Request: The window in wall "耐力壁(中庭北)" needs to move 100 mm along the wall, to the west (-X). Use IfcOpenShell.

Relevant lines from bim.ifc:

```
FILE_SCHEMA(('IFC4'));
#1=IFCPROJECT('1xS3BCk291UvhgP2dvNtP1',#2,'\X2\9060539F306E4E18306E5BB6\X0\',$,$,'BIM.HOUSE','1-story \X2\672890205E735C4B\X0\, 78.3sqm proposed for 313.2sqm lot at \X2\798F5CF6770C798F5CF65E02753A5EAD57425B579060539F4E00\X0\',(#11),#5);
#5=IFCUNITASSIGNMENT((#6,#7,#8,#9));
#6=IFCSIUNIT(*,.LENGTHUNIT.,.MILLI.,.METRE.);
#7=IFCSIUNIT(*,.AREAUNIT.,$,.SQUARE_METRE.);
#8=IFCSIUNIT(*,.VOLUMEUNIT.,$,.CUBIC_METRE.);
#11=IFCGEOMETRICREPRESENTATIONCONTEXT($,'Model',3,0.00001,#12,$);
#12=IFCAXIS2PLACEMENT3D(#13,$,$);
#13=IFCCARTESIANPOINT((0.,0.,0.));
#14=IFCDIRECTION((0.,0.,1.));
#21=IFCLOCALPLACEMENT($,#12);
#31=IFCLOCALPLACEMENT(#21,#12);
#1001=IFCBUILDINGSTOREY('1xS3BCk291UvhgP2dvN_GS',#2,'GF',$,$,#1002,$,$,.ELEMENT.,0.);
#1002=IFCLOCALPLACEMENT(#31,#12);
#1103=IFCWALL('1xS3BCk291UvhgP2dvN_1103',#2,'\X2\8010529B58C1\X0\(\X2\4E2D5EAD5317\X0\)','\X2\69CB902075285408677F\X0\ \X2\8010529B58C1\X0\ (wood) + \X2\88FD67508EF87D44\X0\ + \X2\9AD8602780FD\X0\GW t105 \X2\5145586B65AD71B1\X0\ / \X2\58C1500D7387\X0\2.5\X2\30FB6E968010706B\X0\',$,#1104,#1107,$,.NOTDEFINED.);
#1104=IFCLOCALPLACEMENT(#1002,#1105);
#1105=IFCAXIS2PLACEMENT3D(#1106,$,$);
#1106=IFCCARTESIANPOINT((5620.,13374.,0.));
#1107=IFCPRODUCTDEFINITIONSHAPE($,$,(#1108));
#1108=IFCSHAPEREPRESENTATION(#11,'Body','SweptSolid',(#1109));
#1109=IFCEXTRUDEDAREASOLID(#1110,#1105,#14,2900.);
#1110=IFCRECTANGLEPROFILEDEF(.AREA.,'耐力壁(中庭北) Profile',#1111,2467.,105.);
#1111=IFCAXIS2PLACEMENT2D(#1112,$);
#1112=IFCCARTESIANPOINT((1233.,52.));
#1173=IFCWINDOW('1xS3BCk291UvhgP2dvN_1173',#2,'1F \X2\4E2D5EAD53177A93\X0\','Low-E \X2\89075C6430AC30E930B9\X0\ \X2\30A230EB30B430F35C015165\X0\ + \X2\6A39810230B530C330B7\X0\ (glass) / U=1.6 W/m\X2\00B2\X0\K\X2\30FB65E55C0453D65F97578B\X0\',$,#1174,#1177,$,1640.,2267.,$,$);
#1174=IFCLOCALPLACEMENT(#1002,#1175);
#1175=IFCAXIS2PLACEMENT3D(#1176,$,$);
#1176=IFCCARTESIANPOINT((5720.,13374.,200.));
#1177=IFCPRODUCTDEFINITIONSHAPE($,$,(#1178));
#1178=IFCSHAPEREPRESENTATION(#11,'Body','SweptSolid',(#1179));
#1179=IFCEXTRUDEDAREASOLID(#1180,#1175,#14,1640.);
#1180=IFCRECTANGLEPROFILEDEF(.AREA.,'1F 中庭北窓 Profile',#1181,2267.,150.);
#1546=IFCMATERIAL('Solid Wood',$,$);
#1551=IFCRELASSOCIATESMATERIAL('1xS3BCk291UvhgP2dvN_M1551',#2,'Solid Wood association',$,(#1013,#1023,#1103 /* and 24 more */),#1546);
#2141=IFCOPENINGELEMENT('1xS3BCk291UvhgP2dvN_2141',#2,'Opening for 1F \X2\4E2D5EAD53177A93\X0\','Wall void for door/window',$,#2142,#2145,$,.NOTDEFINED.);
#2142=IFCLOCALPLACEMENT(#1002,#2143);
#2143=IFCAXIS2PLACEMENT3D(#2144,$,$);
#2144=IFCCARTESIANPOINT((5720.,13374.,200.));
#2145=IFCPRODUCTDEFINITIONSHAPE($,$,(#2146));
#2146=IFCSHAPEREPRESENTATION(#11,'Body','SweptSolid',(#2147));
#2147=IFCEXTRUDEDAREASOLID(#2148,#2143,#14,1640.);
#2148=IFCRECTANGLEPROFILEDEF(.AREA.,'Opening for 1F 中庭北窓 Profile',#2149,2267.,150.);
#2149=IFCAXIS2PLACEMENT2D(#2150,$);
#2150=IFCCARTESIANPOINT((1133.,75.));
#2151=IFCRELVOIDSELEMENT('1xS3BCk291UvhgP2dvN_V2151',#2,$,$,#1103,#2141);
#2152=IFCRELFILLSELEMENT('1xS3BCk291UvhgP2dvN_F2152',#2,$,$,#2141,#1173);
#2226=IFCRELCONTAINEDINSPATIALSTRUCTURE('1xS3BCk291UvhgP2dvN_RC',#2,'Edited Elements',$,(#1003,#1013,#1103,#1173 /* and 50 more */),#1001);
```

```python
import ifcopenshell
import ifcopenshell.api.geometry
import ifcopenshell.util.placement
import ifcopenshell.util.unit

model = ifcopenshell.open("bim.ifc")
unit_scale = ifcopenshell.util.unit.calculate_unit_scale(model)

window = model.by_guid("1xS3BCk291UvhgP2dvN_1173")
opening = window.FillsVoids[0].RelatingOpeningElement
wall = opening.VoidsElements[0].RelatingBuildingElement

wall_matrix = ifcopenshell.util.placement.get_local_placement(wall.ObjectPlacement)
shift = wall_matrix[:3, 0] * -0.1 / unit_scale
before = ifcopenshell.util.placement.get_local_placement(window.ObjectPlacement)[:3, 3].copy()

# The window is not placed relative to its opening, so move both.
for product in (opening, window):
    matrix = ifcopenshell.util.placement.get_local_placement(product.ObjectPlacement)
    matrix[:3, 3] += shift
    ifcopenshell.api.geometry.edit_object_placement(model, product=product, matrix=matrix, is_si=False)

after = ifcopenshell.util.placement.get_local_placement(window.ObjectPlacement)[:3, 3]
print("window moved by", (after - before).round(3) + 0.0)

model.write("bim_rev.ifc")
```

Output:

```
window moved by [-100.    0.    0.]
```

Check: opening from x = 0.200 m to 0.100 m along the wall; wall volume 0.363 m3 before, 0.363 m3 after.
